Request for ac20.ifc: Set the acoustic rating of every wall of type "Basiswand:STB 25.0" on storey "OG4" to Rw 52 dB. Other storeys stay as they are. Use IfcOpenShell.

First a look at what the model holds.

```python
import ifcopenshell
import ifcopenshell.util.element

model = ifcopenshell.open("ac20.ifc")
print(model.schema)
storey = next(s for s in model.by_type("IfcBuildingStorey") if s.Name == "OG4")
walls = [e for e in ifcopenshell.util.element.get_decomposition(storey) if e.is_a("IfcWall")]
seen = {}
for e in walls:
    element_type = ifcopenshell.util.element.get_type(e)
    key = (element_type.Name if element_type != e and element_type else None, ifcopenshell.util.element.get_pset(e, "Pset_WallCommon", "AcousticRating"))
    seen[key] = seen.get(key, 0) + 1
for (name, value), count in sorted(seen.items(), key=str):
    print(count, "x", name, "|", value)
```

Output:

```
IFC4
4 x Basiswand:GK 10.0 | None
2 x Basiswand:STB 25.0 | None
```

```python
import ifcopenshell
import ifcopenshell.api.pset
import ifcopenshell.util.element

model = ifcopenshell.open("ac20.ifc")

storey = next(s for s in model.by_type("IfcBuildingStorey") if s.Name == "OG4")
walls = [e for e in ifcopenshell.util.element.get_decomposition(storey) if e.is_a("IfcWall")]

count = 0
for e in walls:
    element_type = ifcopenshell.util.element.get_type(e)
    if element_type in (None, e) or element_type.Name != "Basiswand:STB 25.0":
        continue
    # add_pset returns the element's existing set when there is one.
    pset = ifcopenshell.api.pset.add_pset(model, product=e, name="Pset_WallCommon")
    ifcopenshell.api.pset.edit_pset(model, pset=pset, properties={"AcousticRating": "Rw 52 dB"})
    count += 1

print(count, "walls updated")

model.write("ac20-out.ifc")
```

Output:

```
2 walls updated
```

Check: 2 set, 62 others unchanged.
